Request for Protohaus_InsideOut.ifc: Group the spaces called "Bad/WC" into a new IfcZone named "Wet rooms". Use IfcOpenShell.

First a look at what the model holds.

```python
import ifcopenshell

model = ifcopenshell.open("Protohaus_InsideOut.ifc")
print(model.schema)
seen = {}
for space in model.by_type("IfcSpace"):
    seen[space.LongName] = seen.get(space.LongName, 0) + 1
for name, count in sorted(seen.items(), key=str):
    print(count, "x", name)
print("zones:", [z.Name for z in model.by_type("IfcZone")][:20])
```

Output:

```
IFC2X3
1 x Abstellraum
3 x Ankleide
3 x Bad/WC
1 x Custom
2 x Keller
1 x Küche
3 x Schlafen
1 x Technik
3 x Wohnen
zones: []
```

```python
import ifcopenshell
import ifcopenshell.api.group
import ifcopenshell.api.root

model = ifcopenshell.open("Protohaus_InsideOut.ifc")

names = {"Bad/WC"}
spaces = [s for s in model.by_type("IfcSpace") if s.LongName in names]

zone = ifcopenshell.api.root.create_entity(model, ifc_class="IfcZone", name="Wet rooms")
ifcopenshell.api.group.assign_group(model, products=spaces, group=zone)
print(len(spaces), "spaces in", zone.Name)

model.write("Protohaus_InsideOut-out.ifc")
```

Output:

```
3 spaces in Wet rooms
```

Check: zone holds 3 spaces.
